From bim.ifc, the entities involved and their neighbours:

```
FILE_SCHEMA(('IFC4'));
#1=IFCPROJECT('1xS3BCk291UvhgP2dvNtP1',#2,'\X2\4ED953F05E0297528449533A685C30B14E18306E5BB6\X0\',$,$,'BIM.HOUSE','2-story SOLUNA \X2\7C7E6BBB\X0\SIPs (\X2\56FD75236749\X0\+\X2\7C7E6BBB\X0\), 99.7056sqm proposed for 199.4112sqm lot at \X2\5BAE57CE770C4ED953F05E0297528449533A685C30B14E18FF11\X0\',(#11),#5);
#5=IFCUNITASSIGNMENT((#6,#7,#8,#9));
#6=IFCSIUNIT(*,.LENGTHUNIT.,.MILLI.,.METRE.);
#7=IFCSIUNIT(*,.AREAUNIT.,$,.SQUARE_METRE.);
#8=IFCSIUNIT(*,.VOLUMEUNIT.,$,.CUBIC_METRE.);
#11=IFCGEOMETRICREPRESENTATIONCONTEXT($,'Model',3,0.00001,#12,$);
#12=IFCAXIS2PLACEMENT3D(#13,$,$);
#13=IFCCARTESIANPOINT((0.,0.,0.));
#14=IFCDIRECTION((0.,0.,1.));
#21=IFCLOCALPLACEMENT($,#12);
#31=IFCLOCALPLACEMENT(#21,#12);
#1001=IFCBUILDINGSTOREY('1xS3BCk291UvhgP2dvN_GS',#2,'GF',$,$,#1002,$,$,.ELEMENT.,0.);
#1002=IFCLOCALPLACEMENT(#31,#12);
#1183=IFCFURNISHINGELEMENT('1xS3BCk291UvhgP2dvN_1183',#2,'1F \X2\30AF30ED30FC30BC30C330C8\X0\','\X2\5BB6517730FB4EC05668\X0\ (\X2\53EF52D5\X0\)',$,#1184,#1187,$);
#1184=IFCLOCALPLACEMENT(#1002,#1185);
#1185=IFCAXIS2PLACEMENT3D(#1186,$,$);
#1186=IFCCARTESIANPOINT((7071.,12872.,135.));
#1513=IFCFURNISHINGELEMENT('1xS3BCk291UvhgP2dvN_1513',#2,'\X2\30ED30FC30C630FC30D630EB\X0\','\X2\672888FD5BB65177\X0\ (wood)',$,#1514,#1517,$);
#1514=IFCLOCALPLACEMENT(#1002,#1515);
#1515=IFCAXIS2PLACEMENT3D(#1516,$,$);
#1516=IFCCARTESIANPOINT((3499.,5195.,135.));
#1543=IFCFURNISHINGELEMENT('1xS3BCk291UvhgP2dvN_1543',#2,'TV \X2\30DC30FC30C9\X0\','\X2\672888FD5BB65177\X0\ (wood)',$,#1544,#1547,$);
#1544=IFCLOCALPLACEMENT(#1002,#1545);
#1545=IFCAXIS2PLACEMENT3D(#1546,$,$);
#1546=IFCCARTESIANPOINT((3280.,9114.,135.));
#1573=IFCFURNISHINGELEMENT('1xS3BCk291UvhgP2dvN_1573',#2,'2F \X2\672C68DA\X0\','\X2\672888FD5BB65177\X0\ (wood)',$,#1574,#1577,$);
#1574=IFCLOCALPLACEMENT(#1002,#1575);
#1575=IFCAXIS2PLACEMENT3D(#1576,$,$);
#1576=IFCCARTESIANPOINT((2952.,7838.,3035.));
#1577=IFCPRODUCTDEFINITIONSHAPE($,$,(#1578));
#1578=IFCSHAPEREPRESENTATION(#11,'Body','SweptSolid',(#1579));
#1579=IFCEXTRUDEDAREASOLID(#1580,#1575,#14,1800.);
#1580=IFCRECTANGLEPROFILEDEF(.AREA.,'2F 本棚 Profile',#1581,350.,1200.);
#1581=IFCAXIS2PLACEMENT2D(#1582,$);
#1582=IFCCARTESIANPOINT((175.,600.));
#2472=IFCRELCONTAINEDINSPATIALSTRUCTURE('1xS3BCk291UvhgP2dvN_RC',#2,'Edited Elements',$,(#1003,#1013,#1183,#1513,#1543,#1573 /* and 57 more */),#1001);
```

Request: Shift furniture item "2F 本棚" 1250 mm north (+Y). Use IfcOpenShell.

```python
import ifcopenshell
import ifcopenshell.api.geometry
import ifcopenshell.util.placement

model = ifcopenshell.open("bim.ifc")

item = model.by_id(1573)
matrix = ifcopenshell.util.placement.get_local_placement(item.ObjectPlacement)
matrix[1, 3] += 1250.0
ifcopenshell.api.geometry.edit_object_placement(model, product=item, matrix=matrix, is_si=False)

print(ifcopenshell.util.placement.get_local_placement(item.ObjectPlacement).round(3) + 0.0)

model.write("bim_edited.ifc")
```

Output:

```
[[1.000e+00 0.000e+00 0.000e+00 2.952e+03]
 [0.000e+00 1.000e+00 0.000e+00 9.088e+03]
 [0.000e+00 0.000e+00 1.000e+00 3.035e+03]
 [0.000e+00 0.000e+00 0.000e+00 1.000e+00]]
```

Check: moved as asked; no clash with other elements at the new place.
